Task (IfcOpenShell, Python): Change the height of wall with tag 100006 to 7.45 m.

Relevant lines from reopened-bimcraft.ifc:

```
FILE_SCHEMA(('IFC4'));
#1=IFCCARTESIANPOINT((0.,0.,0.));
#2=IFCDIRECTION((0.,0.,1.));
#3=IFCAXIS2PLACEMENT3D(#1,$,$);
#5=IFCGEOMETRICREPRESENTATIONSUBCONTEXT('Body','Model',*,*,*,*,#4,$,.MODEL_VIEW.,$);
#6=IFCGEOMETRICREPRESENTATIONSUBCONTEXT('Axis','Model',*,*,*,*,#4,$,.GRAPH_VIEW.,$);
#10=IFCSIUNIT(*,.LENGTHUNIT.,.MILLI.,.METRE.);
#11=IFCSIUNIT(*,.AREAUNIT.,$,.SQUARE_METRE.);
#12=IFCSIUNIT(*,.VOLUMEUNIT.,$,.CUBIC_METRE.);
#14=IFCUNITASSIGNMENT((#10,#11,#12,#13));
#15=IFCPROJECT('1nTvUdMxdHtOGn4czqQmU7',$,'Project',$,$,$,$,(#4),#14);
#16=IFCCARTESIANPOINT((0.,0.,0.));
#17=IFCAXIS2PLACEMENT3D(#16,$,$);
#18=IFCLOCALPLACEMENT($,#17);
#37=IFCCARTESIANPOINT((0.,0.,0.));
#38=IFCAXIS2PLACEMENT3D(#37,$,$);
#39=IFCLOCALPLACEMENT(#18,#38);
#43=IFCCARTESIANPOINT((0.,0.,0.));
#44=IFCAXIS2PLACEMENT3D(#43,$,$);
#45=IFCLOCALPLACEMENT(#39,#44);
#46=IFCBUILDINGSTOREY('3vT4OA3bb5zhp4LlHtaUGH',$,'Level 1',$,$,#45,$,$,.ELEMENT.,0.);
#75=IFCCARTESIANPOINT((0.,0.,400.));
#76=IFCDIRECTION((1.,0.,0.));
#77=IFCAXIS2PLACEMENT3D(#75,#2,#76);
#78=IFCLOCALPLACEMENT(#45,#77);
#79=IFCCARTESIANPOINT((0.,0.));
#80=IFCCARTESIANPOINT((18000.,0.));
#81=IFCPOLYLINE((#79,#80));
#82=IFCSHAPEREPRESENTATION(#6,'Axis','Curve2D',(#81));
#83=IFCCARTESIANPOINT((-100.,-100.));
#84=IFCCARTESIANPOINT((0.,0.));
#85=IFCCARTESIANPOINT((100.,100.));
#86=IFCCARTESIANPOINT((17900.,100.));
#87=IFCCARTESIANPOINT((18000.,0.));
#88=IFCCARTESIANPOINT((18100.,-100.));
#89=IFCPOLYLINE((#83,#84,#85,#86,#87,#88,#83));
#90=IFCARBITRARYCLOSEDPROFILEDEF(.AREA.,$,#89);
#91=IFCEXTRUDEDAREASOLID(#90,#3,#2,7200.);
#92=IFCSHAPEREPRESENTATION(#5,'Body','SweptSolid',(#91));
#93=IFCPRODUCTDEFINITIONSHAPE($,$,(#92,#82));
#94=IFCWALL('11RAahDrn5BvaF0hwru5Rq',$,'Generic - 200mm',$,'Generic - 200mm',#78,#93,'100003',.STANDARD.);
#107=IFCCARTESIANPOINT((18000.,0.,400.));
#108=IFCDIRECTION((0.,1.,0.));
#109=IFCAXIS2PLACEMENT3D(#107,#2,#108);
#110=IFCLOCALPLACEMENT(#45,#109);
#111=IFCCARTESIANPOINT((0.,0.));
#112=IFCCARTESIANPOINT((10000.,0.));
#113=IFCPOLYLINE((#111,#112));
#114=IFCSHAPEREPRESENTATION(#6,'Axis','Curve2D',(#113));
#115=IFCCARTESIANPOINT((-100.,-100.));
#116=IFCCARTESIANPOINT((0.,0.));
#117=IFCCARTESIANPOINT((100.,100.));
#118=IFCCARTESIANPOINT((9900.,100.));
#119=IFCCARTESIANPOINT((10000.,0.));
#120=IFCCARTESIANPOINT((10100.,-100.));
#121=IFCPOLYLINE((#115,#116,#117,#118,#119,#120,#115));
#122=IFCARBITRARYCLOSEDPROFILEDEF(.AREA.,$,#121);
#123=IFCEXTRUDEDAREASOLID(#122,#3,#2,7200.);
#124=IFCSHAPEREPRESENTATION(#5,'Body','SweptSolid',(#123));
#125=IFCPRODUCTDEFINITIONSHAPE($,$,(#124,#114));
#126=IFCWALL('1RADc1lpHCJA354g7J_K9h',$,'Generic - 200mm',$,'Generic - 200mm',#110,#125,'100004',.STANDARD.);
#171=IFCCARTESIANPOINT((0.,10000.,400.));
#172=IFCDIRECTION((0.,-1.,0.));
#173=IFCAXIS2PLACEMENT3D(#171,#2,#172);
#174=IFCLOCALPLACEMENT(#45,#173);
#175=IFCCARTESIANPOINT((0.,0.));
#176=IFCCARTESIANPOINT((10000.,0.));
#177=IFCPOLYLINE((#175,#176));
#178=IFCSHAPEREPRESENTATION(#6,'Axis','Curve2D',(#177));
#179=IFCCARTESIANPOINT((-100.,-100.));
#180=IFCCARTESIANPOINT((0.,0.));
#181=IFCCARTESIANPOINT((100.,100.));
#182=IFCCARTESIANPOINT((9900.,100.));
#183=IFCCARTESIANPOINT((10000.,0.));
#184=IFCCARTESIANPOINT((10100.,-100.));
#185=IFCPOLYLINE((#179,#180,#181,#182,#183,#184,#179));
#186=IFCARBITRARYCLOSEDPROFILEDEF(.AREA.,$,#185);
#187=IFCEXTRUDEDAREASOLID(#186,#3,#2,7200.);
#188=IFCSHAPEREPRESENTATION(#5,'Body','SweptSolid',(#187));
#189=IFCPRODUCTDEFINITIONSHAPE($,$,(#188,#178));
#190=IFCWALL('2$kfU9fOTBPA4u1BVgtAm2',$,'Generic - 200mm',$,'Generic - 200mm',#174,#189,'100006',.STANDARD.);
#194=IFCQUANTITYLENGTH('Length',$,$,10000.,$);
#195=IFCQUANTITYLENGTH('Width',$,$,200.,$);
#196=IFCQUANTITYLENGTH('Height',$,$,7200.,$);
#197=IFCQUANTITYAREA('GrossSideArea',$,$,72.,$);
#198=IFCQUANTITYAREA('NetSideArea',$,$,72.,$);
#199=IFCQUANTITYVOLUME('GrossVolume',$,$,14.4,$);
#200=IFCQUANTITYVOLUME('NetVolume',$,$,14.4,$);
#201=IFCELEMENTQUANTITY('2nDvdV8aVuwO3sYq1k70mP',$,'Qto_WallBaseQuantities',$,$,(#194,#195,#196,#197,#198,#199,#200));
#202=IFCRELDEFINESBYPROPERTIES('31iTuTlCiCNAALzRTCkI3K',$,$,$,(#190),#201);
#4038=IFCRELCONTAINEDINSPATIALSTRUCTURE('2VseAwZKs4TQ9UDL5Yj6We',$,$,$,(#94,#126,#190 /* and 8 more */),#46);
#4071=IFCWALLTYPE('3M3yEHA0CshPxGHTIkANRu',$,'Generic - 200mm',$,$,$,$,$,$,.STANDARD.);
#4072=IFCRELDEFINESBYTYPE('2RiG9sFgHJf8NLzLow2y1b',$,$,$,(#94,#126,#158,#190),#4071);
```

```python
import ifcopenshell
import ifcopenshell.api.pset
import ifcopenshell.geom
import ifcopenshell.util.element
import ifcopenshell.util.representation
import ifcopenshell.util.shape
import ifcopenshell.util.unit

model = ifcopenshell.open("reopened-bimcraft.ifc")
unit_scale = ifcopenshell.util.unit.calculate_unit_scale(model)
area_scale = ifcopenshell.util.unit.calculate_unit_scale(model, "AREAUNIT")
volume_scale = ifcopenshell.util.unit.calculate_unit_scale(model, "VOLUMEUNIT")
settings = ifcopenshell.geom.settings()


def volume(element):
    """Net volume in cubic metres, openings subtracted."""
    shape = ifcopenshell.geom.create_shape(settings, element)
    return ifcopenshell.util.shape.get_volume(shape.geometry)


wall = model.by_guid("2$kfU9fOTBPA4u1BVgtAm2")
before = volume(wall)

body = ifcopenshell.util.representation.get_representation(wall, "Model", "Body")
solid = body.Items[0]
old_height = solid.Depth
solid.Depth = 7450.0
after = volume(wall)
thickness = 0.2  # wall thickness in metres

# Update the stored height, areas and volumes.
qto = model.by_id(ifcopenshell.util.element.get_pset(wall, "Qto_WallBaseQuantities", should_inherit=False)["id"])
ifcopenshell.api.pset.edit_qto(model, qto=qto, properties={
    "Height": solid.Depth,
    "GrossSideArea": ifcopenshell.util.element.get_pset(wall, "Qto_WallBaseQuantities", "GrossSideArea") * solid.Depth / old_height,
    "NetSideArea": after / thickness / area_scale,
    "GrossVolume": ifcopenshell.util.element.get_pset(wall, "Qto_WallBaseQuantities", "GrossVolume") * solid.Depth / old_height,
    "NetVolume": after / volume_scale,
})

print(f"height {old_height:g} -> {solid.Depth:g}, volume {before:.3f} -> {after:.3f} m3")

model.write("reopened-bimcraft_v2.ifc")
```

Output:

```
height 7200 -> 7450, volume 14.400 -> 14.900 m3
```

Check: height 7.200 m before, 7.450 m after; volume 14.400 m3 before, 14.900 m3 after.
